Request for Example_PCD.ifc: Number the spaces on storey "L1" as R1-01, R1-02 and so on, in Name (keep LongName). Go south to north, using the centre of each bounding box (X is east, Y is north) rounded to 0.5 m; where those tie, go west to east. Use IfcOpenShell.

First a look at what the model holds.

```python
import ifcopenshell
import ifcopenshell.util.element
import ifcopenshell.util.placement

model = ifcopenshell.open("Example_PCD.ifc")
print(model.schema)
storey = next(s for s in model.by_type("IfcBuildingStorey") if s.Name == "L1")
spaces = [e for e in ifcopenshell.util.element.get_decomposition(storey) if e.is_a("IfcSpace")]
for e in sorted(spaces, key=lambda e: e.id()):
    origin = ifcopenshell.util.placement.get_local_placement(e.ObjectPlacement)[:3, 3]
    print(e.id(), e.Name, e.LongName, origin.round(2) + 0.0, sep=" | ")
```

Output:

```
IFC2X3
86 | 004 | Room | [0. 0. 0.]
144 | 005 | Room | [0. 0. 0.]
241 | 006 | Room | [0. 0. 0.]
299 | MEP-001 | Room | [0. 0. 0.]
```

```python
import ifcopenshell
import ifcopenshell.geom
import ifcopenshell.util.element
import ifcopenshell.util.shape

model = ifcopenshell.open("Example_PCD.ifc")
settings = ifcopenshell.geom.settings()
settings.set("use-world-coords", True)


def centre(element):
    shape = ifcopenshell.geom.create_shape(settings, element)
    return ifcopenshell.util.shape.get_bbox_centroid(shape.geometry)


storey = next(s for s in model.by_type("IfcBuildingStorey") if s.Name == "L1")
spaces = [e for e in ifcopenshell.util.element.get_decomposition(storey) if e.is_a("IfcSpace")]

# Insertion points can sit at a corner or the storey origin, so sort by the geometry (in metres).
centres = {e: centre(e) for e in spaces}
spaces.sort(key=lambda e: (round(centres[e][1] / 0.5), centres[e][0]))

for i, e in enumerate(spaces, start=1):
    number = f"R1-{i:02d}"
    e.Name = number
    print(e.id(), number)

model.write("Example_PCD_edited.ifc")
```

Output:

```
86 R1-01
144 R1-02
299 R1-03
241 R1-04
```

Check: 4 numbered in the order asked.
